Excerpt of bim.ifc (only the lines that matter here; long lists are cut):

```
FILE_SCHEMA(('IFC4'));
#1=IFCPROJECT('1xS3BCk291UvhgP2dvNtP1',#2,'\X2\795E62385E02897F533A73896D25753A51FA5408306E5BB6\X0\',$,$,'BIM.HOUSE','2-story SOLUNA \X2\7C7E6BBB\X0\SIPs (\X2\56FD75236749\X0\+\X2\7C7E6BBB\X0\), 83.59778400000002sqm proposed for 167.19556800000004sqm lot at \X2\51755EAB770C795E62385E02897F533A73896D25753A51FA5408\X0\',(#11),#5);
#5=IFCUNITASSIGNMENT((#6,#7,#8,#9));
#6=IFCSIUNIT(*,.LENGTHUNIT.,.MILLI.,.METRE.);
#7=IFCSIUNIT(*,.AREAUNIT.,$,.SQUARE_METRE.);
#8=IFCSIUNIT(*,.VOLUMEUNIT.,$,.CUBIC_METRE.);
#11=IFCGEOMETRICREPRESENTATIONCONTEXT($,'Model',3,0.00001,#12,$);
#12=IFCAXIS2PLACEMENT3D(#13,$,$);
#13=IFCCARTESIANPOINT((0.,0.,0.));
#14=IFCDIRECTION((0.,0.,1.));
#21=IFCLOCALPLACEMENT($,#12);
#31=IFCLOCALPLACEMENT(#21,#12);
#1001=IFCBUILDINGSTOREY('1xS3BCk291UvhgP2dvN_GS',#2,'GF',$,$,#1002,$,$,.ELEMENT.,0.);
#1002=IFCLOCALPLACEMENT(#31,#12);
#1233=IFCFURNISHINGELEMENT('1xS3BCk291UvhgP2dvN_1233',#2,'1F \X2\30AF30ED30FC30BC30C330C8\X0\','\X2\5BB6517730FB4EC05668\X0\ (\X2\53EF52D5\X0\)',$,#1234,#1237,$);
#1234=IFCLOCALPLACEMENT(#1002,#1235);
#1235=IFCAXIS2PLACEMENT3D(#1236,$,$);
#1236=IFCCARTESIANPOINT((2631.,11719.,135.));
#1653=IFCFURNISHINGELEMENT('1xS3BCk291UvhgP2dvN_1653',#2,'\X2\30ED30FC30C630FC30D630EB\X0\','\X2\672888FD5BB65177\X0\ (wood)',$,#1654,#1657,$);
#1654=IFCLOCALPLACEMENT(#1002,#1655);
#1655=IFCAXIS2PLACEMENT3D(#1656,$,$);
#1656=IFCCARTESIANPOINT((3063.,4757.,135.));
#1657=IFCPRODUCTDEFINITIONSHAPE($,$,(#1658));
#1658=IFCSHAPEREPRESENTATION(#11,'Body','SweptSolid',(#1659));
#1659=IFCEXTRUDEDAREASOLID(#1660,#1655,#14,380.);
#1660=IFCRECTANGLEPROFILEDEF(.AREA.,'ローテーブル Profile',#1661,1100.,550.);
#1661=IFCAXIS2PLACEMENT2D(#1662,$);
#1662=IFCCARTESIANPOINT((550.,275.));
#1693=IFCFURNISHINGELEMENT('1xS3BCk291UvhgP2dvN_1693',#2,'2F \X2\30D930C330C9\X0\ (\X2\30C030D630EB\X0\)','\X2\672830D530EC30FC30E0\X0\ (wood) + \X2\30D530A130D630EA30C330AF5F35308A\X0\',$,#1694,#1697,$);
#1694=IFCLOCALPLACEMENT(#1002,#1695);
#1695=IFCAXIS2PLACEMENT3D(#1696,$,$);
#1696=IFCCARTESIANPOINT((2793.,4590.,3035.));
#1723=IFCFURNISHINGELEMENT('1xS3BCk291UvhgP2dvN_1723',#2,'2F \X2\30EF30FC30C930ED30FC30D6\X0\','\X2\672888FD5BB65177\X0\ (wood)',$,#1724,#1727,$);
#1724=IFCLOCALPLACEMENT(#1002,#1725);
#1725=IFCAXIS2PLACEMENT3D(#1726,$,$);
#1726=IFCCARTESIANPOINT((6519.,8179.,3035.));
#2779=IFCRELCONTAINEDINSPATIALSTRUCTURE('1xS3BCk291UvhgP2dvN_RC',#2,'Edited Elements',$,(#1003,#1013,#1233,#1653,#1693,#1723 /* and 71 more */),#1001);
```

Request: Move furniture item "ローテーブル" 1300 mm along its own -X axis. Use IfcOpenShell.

```python
import ifcopenshell
import ifcopenshell.api.geometry
import ifcopenshell.util.placement

model = ifcopenshell.open("bim.ifc")

item = model.by_guid("1xS3BCk291UvhgP2dvN_1653")
matrix = ifcopenshell.util.placement.get_local_placement(item.ObjectPlacement)
matrix[:3, 3] -= matrix[:3, 0] * 1300.0
ifcopenshell.api.geometry.edit_object_placement(model, product=item, matrix=matrix, is_si=False)

print(ifcopenshell.util.placement.get_local_placement(item.ObjectPlacement).round(3) + 0.0)

model.write("bim_updated.ifc")
```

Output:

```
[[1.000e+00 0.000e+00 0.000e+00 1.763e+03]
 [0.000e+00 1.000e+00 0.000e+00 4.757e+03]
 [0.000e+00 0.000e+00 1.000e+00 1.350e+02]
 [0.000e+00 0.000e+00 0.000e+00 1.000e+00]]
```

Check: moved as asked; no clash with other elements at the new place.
